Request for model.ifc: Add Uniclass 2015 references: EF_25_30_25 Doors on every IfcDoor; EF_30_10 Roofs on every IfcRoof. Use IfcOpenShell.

First a look at what the model holds.

```python
import ifcopenshell

model = ifcopenshell.open("model.ifc")
print(model.schema)
print("classifications:", [c.Name for c in model.by_type("IfcClassification")])
for ifc_class in ("IfcDoor", "IfcRoof", "IfcStair", "IfcWall", "IfcWindow"):
    print(ifc_class, len(model.by_type(ifc_class)))
```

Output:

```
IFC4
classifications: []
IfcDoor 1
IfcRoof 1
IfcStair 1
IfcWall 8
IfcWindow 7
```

```python
import ifcopenshell
import ifcopenshell.api.classification

model = ifcopenshell.open("model.ifc")

system = ifcopenshell.api.classification.add_classification(model, classification="Uniclass 2015")

codes = {
    "IfcDoor": ("EF_25_30_25", "Doors"),
    "IfcRoof": ("EF_30_10", "Roofs"),
}
for ifc_class, (code, name) in codes.items():
    products = model.by_type(ifc_class)
    ifcopenshell.api.classification.add_reference(
        model, products=products, classification=system, identification=code, name=name
    )
    print(code, len(products))

model.write("model_v2.ifc")
```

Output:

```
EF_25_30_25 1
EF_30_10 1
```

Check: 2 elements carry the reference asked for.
